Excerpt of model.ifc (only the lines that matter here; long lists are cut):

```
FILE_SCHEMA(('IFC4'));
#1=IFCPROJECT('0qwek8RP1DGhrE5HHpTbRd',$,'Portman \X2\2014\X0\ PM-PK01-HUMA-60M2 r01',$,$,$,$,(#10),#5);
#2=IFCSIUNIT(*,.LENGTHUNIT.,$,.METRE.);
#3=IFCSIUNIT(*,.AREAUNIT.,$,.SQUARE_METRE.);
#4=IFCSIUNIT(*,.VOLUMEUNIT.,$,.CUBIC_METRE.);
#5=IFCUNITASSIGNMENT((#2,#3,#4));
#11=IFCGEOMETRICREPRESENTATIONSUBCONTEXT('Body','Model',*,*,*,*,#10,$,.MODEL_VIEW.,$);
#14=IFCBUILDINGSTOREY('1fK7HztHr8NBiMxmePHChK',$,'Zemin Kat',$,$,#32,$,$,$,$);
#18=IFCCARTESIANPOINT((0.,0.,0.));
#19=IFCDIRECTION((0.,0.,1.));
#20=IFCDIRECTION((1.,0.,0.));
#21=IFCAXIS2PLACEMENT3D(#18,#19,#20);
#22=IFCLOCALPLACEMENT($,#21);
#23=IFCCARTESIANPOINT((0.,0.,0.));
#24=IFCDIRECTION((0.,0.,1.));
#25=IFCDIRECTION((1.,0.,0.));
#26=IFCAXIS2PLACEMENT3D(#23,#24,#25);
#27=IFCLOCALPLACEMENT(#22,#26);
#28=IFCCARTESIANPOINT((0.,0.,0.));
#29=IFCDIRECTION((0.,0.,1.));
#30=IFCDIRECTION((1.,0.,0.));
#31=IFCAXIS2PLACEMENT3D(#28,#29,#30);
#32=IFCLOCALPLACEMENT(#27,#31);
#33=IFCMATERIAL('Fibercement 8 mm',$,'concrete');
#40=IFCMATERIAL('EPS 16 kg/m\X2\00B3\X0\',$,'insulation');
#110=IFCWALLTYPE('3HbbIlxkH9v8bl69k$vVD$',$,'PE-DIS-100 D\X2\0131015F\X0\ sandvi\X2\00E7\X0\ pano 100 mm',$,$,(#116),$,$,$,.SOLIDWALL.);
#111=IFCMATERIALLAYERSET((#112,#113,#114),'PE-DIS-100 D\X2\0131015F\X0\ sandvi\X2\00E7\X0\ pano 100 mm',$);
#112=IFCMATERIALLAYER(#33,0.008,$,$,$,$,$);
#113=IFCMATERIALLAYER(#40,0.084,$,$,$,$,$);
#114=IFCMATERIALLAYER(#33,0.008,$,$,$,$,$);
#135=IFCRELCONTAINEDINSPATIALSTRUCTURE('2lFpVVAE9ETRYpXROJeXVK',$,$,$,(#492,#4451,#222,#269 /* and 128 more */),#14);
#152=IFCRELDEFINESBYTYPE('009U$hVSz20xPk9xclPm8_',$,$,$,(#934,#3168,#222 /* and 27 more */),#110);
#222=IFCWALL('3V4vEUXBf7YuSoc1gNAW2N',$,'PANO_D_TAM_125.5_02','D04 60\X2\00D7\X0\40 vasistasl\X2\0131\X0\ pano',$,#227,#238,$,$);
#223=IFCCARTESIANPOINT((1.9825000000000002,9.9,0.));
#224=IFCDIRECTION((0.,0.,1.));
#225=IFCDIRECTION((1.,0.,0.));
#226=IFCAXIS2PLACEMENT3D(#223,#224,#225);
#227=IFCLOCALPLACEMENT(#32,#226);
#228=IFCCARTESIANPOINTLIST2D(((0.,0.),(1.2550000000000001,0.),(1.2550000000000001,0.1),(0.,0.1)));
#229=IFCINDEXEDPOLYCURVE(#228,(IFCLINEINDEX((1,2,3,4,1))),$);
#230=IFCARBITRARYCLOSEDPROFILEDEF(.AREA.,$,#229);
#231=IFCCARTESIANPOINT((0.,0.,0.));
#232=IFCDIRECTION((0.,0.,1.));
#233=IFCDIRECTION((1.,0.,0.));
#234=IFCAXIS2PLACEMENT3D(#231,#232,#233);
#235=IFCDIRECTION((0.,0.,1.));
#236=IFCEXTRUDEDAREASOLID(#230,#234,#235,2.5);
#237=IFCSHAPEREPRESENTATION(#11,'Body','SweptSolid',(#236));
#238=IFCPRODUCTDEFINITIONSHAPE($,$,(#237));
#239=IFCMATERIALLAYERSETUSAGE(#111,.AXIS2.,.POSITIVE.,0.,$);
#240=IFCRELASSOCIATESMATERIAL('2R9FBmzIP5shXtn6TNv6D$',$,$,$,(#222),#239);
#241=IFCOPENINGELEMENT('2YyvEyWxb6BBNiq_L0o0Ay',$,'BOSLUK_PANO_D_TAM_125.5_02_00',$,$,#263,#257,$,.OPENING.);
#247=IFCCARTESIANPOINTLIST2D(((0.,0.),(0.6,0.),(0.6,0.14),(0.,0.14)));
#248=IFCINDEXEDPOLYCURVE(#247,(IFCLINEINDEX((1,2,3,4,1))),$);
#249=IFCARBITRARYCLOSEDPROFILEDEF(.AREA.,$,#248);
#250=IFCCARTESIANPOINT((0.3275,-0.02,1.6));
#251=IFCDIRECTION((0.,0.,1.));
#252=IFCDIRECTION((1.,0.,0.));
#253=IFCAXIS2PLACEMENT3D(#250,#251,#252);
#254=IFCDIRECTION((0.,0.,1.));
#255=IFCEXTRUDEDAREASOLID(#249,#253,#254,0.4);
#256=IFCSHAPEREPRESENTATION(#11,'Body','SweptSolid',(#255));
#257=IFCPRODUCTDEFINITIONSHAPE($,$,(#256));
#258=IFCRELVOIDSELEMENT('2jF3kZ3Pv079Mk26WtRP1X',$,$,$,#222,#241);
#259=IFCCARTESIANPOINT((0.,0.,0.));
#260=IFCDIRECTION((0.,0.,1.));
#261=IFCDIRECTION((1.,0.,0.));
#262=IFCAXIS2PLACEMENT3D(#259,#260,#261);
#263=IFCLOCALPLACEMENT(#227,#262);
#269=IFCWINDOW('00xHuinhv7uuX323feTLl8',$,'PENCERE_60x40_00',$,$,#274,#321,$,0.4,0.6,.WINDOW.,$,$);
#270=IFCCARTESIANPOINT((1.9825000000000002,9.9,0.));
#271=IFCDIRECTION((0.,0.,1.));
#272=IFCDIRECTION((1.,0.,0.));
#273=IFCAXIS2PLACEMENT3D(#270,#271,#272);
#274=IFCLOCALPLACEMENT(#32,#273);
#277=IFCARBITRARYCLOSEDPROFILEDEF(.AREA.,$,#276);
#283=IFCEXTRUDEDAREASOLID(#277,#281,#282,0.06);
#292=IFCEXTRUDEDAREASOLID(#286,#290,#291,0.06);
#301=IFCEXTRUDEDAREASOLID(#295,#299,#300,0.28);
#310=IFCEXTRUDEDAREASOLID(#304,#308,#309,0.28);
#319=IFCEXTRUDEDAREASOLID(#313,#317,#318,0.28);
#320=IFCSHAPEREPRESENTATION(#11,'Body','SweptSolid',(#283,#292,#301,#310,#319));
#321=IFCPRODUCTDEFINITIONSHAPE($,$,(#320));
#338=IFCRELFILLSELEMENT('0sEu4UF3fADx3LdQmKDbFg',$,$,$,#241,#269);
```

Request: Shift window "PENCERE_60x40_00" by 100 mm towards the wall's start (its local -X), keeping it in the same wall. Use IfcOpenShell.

```python
import ifcopenshell
import ifcopenshell.api.geometry
import ifcopenshell.util.placement
import ifcopenshell.util.unit

model = ifcopenshell.open("model.ifc")
unit_scale = ifcopenshell.util.unit.calculate_unit_scale(model)

window = model.by_id(269)
opening = window.FillsVoids[0].RelatingOpeningElement
wall = opening.VoidsElements[0].RelatingBuildingElement

wall_matrix = ifcopenshell.util.placement.get_local_placement(wall.ObjectPlacement)
shift = wall_matrix[:3, 0] * -0.1 / unit_scale
before = ifcopenshell.util.placement.get_local_placement(window.ObjectPlacement)[:3, 3].copy()

# The window is not placed relative to its opening, so move both.
for product in (opening, window):
    matrix = ifcopenshell.util.placement.get_local_placement(product.ObjectPlacement)
    matrix[:3, 3] += shift
    ifcopenshell.api.geometry.edit_object_placement(model, product=product, matrix=matrix, is_si=False)

after = ifcopenshell.util.placement.get_local_placement(window.ObjectPlacement)[:3, 3]
print("window moved by", (after - before).round(3) + 0.0)

model.write("model_rev.ifc")
```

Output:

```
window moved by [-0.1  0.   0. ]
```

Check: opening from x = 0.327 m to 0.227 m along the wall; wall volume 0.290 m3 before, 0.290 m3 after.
